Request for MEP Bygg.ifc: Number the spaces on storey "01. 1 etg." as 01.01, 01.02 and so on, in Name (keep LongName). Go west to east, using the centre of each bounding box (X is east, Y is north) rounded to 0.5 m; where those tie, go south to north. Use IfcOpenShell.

First a look at what the model holds.

```python
import ifcopenshell
import ifcopenshell.util.element
import ifcopenshell.util.placement

model = ifcopenshell.open("MEP Bygg.ifc")
print(model.schema)
storey = next(s for s in model.by_type("IfcBuildingStorey") if s.Name == "01. 1 etg.")
spaces = [e for e in ifcopenshell.util.element.get_decomposition(storey) if e.is_a("IfcSpace")]
for e in sorted(spaces, key=lambda e: e.id()):
    origin = ifcopenshell.util.placement.get_local_placement(e.ObjectPlacement)[:3, 3]
    print(e.id(), e.Name, e.LongName, origin.round(2) + 0.0, sep=" | ")
```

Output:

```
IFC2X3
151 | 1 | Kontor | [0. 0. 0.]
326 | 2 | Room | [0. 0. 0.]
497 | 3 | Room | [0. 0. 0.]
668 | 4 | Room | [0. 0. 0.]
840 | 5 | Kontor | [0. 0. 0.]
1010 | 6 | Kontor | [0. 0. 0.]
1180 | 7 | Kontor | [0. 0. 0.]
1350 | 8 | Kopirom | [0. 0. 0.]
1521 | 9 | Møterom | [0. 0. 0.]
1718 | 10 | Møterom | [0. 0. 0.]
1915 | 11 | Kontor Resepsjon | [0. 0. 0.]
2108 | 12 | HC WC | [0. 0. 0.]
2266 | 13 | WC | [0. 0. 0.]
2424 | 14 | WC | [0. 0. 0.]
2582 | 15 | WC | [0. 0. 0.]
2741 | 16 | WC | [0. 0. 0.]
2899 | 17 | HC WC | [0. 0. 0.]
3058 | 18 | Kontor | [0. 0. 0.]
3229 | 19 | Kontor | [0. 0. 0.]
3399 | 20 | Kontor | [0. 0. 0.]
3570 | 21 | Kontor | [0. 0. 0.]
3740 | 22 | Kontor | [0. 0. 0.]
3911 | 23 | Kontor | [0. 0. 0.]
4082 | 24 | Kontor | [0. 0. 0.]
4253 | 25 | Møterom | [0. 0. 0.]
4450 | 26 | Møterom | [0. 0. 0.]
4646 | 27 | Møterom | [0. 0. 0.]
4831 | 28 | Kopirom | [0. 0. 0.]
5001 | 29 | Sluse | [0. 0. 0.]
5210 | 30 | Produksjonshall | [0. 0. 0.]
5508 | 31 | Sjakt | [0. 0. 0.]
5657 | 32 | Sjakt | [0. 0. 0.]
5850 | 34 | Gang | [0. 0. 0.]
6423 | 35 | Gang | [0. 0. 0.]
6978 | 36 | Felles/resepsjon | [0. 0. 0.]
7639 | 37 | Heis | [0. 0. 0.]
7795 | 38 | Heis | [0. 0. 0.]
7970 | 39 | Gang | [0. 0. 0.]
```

```python
import ifcopenshell
import ifcopenshell.geom
import ifcopenshell.util.element
import ifcopenshell.util.shape

model = ifcopenshell.open("MEP Bygg.ifc")
settings = ifcopenshell.geom.settings()
settings.set("use-world-coords", True)


def centre(element):
    shape = ifcopenshell.geom.create_shape(settings, element)
    return ifcopenshell.util.shape.get_bbox_centroid(shape.geometry)


storey = next(s for s in model.by_type("IfcBuildingStorey") if s.Name == "01. 1 etg.")
spaces = [e for e in ifcopenshell.util.element.get_decomposition(storey) if e.is_a("IfcSpace")]

# Insertion points can sit at a corner or the storey origin, so sort by the geometry (in metres).
centres = {e: centre(e) for e in spaces}
spaces.sort(key=lambda e: (round(centres[e][0] / 0.5), centres[e][1]))

for i, e in enumerate(spaces, start=1):
    number = f"01.{i:02d}"
    e.Name = number
    print(e.id(), number)

model.write("MEP Bygg_updated.ifc")
```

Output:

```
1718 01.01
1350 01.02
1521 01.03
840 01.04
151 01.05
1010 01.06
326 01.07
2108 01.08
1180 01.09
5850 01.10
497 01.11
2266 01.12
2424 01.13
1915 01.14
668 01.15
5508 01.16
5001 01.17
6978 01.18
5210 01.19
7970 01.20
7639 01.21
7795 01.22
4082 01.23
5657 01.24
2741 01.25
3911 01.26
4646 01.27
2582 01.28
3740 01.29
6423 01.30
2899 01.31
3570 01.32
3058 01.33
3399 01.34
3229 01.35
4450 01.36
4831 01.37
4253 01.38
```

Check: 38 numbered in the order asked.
